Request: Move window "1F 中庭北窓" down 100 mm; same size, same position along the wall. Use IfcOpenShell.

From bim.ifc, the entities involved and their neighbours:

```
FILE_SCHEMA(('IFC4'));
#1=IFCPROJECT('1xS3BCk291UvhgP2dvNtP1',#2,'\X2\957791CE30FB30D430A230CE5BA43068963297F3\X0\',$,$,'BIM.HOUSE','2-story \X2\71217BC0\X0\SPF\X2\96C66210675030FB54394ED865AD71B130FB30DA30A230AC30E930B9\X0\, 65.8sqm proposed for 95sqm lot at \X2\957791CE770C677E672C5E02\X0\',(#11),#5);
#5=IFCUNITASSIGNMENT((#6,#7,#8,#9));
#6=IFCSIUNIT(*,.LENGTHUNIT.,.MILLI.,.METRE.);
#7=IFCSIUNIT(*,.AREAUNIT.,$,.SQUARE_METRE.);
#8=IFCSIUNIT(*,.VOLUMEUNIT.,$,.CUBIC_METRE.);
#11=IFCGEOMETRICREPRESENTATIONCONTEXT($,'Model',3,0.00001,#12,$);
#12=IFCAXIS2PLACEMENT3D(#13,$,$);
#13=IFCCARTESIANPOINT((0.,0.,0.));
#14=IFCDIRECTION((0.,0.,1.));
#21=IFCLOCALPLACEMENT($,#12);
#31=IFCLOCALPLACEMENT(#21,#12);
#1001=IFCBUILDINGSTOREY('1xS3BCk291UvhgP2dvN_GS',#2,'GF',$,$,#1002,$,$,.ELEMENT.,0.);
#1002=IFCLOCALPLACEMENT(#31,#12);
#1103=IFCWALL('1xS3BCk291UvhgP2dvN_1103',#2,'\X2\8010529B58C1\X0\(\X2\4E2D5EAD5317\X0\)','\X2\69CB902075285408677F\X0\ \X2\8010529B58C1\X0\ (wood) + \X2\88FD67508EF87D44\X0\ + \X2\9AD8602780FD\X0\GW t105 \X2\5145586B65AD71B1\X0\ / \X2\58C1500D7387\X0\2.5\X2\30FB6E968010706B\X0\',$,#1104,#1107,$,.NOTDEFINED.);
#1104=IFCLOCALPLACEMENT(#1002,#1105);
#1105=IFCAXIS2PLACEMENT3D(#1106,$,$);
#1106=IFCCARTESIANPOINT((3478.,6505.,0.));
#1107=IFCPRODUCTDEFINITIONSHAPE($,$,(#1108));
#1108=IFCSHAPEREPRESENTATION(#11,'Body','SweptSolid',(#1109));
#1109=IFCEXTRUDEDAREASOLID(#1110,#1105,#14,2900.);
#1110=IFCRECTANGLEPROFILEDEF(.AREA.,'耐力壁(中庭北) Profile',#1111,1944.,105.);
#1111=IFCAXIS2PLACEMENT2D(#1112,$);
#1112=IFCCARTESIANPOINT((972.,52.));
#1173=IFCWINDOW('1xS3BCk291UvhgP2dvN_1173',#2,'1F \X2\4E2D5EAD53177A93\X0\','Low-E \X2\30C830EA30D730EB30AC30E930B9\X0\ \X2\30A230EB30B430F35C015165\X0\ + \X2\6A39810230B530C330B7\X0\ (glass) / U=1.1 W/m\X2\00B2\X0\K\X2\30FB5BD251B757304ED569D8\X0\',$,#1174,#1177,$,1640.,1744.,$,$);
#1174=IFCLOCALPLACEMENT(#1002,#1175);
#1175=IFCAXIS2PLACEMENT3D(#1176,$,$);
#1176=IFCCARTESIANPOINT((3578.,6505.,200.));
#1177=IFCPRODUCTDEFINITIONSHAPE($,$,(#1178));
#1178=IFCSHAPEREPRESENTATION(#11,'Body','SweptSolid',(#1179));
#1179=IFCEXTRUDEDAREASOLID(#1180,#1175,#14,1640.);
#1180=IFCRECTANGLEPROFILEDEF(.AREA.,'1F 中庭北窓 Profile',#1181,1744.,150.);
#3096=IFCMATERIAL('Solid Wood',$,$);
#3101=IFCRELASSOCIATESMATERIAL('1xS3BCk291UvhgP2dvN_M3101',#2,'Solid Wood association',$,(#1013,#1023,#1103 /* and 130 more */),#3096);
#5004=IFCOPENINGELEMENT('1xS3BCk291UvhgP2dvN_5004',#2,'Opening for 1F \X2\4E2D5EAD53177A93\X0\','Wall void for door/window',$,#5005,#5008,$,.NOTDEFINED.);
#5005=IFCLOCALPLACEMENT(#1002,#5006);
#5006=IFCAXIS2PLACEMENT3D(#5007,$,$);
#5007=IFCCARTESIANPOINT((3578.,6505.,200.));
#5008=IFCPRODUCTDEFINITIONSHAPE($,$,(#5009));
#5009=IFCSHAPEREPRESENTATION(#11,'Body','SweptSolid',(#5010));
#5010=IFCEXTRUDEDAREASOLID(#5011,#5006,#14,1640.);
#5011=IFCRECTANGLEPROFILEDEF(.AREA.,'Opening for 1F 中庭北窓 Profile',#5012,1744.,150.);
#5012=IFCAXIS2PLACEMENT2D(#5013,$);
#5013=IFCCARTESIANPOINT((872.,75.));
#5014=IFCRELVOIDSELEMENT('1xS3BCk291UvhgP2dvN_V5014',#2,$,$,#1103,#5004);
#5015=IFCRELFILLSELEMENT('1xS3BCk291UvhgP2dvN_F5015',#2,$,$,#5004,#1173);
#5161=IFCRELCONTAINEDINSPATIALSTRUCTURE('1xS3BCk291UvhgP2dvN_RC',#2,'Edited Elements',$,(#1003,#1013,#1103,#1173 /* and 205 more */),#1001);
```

```python
import numpy as np
import ifcopenshell
import ifcopenshell.api.geometry
import ifcopenshell.util.placement
import ifcopenshell.util.unit

model = ifcopenshell.open("bim.ifc")
unit_scale = ifcopenshell.util.unit.calculate_unit_scale(model)

window = model.by_guid("1xS3BCk291UvhgP2dvN_1173")
opening = window.FillsVoids[0].RelatingOpeningElement
dz = -0.1 / unit_scale

shift = np.array([0.0, 0.0, dz])
# The window is not placed relative to its opening, so move both.
for product in (opening, window):
    matrix = ifcopenshell.util.placement.get_local_placement(product.ObjectPlacement)
    matrix[:3, 3] += shift
    ifcopenshell.api.geometry.edit_object_placement(model, product=product, matrix=matrix, is_si=False)

print(f"moved by {dz * unit_scale:+.3f} m")

model.write("bim_updated.ifc")
```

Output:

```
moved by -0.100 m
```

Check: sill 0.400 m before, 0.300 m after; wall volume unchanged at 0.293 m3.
